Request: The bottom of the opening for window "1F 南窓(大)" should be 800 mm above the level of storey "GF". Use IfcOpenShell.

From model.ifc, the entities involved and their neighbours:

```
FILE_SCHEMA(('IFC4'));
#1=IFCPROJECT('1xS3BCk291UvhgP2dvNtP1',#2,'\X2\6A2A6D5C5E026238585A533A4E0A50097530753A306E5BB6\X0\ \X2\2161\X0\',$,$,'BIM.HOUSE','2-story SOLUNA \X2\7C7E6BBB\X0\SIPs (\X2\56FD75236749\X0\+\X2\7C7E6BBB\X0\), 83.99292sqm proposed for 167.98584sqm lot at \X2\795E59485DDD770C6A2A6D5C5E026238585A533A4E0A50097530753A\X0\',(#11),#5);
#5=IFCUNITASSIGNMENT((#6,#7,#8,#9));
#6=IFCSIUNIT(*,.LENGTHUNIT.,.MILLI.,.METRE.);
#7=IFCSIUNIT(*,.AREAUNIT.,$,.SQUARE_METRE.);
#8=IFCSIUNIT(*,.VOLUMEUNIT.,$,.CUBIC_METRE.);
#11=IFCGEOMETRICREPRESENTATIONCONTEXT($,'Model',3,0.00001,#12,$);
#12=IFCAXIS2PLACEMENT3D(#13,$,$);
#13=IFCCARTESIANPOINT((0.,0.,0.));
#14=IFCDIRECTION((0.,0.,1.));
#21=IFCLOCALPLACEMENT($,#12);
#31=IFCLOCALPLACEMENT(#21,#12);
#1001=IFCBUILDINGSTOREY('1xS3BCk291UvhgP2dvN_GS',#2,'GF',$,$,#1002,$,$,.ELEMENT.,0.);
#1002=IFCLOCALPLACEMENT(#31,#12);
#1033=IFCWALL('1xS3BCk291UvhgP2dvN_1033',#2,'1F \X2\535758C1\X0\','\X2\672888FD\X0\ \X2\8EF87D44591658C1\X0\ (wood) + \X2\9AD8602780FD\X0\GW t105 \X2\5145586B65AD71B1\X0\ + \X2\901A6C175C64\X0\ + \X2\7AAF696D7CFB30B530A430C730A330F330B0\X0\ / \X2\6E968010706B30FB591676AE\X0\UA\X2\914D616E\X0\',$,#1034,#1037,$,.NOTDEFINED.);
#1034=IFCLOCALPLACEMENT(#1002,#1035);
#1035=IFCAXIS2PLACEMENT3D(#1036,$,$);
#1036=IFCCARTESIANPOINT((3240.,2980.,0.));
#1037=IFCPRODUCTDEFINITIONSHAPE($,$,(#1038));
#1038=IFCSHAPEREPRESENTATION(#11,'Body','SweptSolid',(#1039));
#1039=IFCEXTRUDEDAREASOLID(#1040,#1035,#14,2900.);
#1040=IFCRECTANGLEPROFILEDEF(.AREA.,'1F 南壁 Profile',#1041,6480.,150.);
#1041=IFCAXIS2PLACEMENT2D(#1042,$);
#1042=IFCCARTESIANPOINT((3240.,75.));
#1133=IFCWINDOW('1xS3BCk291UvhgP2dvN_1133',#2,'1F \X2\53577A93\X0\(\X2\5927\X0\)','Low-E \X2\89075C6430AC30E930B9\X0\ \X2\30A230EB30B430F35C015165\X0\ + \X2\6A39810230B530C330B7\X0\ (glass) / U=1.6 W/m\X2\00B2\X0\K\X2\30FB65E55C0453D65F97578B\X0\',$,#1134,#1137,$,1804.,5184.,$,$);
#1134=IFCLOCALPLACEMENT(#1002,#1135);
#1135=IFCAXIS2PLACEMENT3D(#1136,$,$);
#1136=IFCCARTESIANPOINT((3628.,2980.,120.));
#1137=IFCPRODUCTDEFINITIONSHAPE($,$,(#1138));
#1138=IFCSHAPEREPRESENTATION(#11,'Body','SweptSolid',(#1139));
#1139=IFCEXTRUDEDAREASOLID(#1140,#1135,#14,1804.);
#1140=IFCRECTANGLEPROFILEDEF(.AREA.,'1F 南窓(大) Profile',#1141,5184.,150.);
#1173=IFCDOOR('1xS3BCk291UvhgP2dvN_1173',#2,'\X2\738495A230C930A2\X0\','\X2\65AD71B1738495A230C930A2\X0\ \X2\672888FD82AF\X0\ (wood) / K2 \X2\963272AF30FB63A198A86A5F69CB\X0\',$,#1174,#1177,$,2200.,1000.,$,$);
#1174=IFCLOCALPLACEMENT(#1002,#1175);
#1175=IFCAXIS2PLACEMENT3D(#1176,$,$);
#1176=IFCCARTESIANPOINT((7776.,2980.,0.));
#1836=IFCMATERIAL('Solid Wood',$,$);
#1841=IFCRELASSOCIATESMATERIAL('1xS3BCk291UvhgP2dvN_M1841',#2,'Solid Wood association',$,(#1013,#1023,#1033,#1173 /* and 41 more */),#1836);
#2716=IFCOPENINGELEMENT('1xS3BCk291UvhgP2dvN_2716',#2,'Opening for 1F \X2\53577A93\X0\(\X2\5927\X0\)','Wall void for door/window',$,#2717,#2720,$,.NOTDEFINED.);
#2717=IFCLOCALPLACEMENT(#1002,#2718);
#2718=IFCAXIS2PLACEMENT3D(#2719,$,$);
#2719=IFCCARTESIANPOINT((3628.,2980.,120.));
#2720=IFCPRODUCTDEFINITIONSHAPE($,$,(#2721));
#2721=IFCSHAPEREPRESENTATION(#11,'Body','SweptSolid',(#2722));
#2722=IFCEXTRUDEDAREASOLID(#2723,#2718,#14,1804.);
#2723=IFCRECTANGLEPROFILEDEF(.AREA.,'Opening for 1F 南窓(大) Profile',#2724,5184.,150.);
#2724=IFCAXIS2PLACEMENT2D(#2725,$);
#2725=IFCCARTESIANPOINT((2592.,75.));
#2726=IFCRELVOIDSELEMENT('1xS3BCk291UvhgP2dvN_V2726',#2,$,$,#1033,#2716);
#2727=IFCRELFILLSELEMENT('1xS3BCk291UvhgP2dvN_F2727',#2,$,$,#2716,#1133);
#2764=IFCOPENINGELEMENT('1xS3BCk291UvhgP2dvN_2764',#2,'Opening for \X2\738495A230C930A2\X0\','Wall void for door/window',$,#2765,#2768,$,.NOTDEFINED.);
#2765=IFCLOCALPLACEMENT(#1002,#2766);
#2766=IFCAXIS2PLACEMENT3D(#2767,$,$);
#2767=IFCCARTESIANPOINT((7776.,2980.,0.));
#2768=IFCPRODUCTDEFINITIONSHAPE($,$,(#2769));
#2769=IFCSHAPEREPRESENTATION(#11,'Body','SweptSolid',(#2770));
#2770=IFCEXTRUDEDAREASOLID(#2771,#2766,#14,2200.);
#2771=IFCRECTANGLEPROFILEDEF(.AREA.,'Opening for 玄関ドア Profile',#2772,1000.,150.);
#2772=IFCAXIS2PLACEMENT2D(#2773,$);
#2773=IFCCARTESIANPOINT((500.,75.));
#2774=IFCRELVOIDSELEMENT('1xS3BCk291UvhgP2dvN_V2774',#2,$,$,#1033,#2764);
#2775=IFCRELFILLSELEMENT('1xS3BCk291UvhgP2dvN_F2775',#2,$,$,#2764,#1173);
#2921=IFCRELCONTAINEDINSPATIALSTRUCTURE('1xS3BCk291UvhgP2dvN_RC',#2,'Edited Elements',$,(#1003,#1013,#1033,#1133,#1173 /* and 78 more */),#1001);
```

```python
import numpy as np
import ifcopenshell
import ifcopenshell.api.geometry
import ifcopenshell.geom
import ifcopenshell.util.element
import ifcopenshell.util.placement
import ifcopenshell.util.shape
import ifcopenshell.util.unit

model = ifcopenshell.open("model.ifc")
unit_scale = ifcopenshell.util.unit.calculate_unit_scale(model)

window = model.by_guid("1xS3BCk291UvhgP2dvN_1133")
opening = window.FillsVoids[0].RelatingOpeningElement
storey = ifcopenshell.util.element.get_container(window, ifc_class="IfcBuildingStorey")
level = ifcopenshell.util.placement.get_local_placement(storey.ObjectPlacement)[2, 3]

# The opening's origin need not be at the sill, so measure its lowest point.
shape = ifcopenshell.geom.create_shape(ifcopenshell.geom.settings(), opening)
bottom = ifcopenshell.util.shape.get_shape_bottom_elevation(shape, shape.geometry) / unit_scale
dz = level + 800.0 - bottom

shift = np.array([0.0, 0.0, dz])
# The window is not placed relative to its opening, so move both.
for product in (opening, window):
    matrix = ifcopenshell.util.placement.get_local_placement(product.ObjectPlacement)
    matrix[:3, 3] += shift
    ifcopenshell.api.geometry.edit_object_placement(model, product=product, matrix=matrix, is_si=False)

print(f"moved by {dz * unit_scale:+.3f} m")

model.write("model_edited.ifc")
```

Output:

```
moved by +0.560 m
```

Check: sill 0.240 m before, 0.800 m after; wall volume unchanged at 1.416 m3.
